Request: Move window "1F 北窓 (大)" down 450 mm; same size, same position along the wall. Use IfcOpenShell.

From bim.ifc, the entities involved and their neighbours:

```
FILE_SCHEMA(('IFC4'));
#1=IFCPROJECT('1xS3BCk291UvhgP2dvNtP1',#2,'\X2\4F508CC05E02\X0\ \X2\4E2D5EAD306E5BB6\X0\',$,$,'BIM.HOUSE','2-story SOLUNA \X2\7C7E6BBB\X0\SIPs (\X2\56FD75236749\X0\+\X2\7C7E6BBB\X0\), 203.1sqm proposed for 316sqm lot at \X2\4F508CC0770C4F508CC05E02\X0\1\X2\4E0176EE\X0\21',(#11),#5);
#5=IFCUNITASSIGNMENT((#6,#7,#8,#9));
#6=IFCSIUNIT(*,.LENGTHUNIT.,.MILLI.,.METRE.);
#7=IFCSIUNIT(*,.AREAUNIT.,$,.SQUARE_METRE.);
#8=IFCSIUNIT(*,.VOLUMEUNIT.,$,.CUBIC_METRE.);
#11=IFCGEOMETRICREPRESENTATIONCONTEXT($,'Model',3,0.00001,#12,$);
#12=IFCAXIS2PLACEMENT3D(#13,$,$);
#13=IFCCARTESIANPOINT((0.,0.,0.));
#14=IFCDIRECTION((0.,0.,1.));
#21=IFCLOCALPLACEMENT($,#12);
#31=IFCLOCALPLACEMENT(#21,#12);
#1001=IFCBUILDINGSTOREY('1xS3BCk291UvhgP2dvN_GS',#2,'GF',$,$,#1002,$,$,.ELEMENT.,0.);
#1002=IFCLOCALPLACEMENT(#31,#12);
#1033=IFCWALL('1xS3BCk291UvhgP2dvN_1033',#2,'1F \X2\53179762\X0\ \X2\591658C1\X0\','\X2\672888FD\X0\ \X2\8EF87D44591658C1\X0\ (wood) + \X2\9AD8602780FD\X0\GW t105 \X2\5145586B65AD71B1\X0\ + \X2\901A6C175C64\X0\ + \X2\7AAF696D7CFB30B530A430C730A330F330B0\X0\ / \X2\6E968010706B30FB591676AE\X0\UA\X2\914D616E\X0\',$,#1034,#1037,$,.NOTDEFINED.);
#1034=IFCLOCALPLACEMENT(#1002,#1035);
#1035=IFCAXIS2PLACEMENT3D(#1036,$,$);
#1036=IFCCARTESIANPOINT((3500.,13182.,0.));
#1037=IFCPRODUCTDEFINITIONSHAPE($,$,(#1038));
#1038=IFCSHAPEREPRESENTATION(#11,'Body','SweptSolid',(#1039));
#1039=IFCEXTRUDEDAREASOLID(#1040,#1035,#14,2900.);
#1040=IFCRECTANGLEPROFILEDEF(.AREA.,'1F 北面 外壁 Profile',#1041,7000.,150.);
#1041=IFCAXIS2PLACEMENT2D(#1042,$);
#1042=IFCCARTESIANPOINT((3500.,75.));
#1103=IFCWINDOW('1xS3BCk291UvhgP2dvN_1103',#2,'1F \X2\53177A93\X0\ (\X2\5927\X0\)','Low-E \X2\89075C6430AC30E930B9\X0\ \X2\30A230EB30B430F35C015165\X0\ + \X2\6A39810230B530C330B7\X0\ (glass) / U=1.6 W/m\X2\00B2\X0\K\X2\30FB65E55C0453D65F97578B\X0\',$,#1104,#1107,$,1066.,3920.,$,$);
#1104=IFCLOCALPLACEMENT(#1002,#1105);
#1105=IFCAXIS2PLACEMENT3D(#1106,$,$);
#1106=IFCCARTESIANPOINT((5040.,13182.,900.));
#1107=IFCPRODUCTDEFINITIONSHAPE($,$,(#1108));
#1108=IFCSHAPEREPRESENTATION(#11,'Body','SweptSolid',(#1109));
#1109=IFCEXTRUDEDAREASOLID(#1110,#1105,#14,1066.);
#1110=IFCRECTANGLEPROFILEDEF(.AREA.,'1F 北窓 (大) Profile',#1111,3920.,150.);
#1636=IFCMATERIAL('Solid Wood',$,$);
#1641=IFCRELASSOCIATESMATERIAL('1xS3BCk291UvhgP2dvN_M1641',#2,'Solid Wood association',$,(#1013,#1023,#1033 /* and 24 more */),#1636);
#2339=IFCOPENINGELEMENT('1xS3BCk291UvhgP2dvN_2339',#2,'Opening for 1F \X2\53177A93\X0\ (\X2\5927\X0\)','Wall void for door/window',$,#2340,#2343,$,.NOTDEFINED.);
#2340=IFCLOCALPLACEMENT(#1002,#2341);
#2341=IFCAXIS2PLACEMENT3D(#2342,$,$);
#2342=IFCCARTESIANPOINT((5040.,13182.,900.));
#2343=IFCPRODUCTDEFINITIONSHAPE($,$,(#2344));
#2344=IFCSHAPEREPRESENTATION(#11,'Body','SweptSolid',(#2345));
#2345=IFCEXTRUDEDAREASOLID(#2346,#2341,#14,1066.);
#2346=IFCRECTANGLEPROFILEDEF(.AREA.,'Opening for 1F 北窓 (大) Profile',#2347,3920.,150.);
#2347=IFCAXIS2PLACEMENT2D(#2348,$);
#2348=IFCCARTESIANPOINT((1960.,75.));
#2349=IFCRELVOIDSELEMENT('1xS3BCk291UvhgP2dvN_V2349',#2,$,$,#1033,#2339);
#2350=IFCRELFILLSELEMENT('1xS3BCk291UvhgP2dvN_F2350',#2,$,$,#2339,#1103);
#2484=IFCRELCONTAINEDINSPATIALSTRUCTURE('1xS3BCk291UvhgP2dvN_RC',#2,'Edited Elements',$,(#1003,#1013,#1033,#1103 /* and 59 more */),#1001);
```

```python
import numpy as np
import ifcopenshell
import ifcopenshell.api.geometry
import ifcopenshell.util.placement
import ifcopenshell.util.unit

model = ifcopenshell.open("bim.ifc")
unit_scale = ifcopenshell.util.unit.calculate_unit_scale(model)

window = model.by_guid("1xS3BCk291UvhgP2dvN_1103")
opening = window.FillsVoids[0].RelatingOpeningElement
dz = -0.45 / unit_scale

shift = np.array([0.0, 0.0, dz])
# The window is not placed relative to its opening, so move both.
for product in (opening, window):
    matrix = ifcopenshell.util.placement.get_local_placement(product.ObjectPlacement)
    matrix[:3, 3] += shift
    ifcopenshell.api.geometry.edit_object_placement(model, product=product, matrix=matrix, is_si=False)

print(f"moved by {dz * unit_scale:+.3f} m")

model.write("bim_edited.ifc")
```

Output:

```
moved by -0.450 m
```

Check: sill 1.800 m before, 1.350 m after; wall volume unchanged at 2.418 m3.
